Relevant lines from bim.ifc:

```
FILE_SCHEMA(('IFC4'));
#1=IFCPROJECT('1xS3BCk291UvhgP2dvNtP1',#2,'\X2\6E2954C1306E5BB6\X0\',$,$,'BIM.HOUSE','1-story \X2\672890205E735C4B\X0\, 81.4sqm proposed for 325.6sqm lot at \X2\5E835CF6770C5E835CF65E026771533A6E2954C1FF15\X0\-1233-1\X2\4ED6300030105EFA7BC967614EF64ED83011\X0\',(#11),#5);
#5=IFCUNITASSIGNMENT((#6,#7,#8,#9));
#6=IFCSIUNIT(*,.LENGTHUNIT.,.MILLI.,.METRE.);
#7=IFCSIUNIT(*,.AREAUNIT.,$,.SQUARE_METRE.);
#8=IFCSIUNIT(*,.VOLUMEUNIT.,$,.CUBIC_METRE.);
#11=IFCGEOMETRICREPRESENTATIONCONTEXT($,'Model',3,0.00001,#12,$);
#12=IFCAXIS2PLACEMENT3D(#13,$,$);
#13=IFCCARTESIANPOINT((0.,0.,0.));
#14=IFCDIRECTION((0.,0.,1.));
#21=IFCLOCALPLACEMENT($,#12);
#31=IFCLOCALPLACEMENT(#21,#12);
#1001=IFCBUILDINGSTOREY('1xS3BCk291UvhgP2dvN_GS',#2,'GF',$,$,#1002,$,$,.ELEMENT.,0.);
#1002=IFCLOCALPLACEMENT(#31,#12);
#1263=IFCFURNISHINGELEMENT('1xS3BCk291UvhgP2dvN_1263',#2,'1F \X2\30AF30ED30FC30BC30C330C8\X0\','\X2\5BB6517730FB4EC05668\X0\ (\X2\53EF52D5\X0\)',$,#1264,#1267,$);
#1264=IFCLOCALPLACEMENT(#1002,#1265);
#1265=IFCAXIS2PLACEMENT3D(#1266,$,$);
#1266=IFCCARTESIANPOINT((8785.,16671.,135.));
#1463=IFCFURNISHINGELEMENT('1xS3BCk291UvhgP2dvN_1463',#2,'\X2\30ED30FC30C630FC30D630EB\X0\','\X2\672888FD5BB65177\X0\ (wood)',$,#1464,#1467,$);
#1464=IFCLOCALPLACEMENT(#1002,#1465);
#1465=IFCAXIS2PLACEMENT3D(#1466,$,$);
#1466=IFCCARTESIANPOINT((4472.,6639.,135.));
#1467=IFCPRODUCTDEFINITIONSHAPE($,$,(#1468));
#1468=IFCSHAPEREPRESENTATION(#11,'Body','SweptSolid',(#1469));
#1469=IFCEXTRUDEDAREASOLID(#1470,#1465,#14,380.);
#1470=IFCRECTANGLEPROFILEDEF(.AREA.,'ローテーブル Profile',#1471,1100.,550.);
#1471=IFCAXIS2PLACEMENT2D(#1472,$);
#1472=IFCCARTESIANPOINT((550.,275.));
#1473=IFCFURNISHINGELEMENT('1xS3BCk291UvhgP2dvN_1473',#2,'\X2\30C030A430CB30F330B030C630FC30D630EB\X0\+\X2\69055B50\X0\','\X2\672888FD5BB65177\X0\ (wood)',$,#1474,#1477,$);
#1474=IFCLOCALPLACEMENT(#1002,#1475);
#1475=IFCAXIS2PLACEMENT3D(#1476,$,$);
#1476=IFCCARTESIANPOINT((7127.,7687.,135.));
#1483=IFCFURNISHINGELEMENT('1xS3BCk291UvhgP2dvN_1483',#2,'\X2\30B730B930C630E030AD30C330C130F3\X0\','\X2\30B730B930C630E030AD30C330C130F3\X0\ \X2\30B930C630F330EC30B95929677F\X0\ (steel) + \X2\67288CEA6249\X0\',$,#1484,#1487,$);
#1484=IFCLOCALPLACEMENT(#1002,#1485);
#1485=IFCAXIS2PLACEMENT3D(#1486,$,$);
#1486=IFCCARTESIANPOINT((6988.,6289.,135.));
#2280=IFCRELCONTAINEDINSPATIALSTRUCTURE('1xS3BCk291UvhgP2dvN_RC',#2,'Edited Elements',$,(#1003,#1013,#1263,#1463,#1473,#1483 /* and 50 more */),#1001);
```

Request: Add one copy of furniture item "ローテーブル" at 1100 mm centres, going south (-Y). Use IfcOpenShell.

```python
import numpy as np
import ifcopenshell
import ifcopenshell.api.geometry
import ifcopenshell.api.root
import ifcopenshell.util.element
import ifcopenshell.util.placement

model = ifcopenshell.open("bim.ifc")


def reuse_history(source, copy):
    """copy_class also copies each property set's owner history, people and application; keep the originals."""
    for rel in copy.IsDefinedBy:
        if rel.is_a("IfcRelDefinesByProperties") and (history := rel.RelatingPropertyDefinition.OwnerHistory):
            rel.RelatingPropertyDefinition.OwnerHistory = source.OwnerHistory
            ifcopenshell.util.element.remove_deep2(model, history)


source = model.by_id(1463)
base = ifcopenshell.util.placement.get_local_placement(source.ObjectPlacement)
step = np.array([0.0, -1.0, 0.0]) * 1100.0

for i in range(1, 2):
    copy = ifcopenshell.api.root.copy_class(model, product=source)
    copy.Representation = ifcopenshell.util.element.copy_deep(
        model, source.Representation, exclude=["IfcGeometricRepresentationContext", "IfcRepresentationMap"]
    )
    reuse_history(source, copy)
    matrix = base.copy()
    matrix[:3, 3] += i * step
    print("added at", matrix[:3, 3].round(3) + 0.0)
    ifcopenshell.api.geometry.edit_object_placement(model, product=copy, matrix=matrix, is_si=False)

model.write("bim_edited.ifc")
```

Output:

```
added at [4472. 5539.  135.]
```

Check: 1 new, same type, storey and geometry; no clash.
